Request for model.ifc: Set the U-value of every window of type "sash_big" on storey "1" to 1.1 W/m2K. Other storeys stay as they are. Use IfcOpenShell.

First a look at what the model holds.

```python
import ifcopenshell
import ifcopenshell.util.element

model = ifcopenshell.open("model.ifc")
print(model.schema)
storey = next(s for s in model.by_type("IfcBuildingStorey") if s.Name == "1")
windows = [e for e in ifcopenshell.util.element.get_decomposition(storey) if e.is_a("IfcWindow")]
seen = {}
for e in windows:
    element_type = ifcopenshell.util.element.get_type(e)
    key = (element_type.Name if element_type != e and element_type else None, ifcopenshell.util.element.get_pset(e, "Pset_WindowCommon", "ThermalTransmittance"))
    seen[key] = seen.get(key, 0) + 1
for (name, value), count in sorted(seen.items(), key=str):
    print(count, "x", name, "|", value)
```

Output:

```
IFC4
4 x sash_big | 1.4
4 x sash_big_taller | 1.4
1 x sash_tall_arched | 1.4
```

```python
import ifcopenshell
import ifcopenshell.api.pset
import ifcopenshell.util.element

model = ifcopenshell.open("model.ifc")

storey = next(s for s in model.by_type("IfcBuildingStorey") if s.Name == "1")
windows = [e for e in ifcopenshell.util.element.get_decomposition(storey) if e.is_a("IfcWindow")]

count = 0
for e in windows:
    element_type = ifcopenshell.util.element.get_type(e)
    if element_type in (None, e) or element_type.Name != "sash_big":
        continue
    # add_pset returns the element's existing set when there is one.
    pset = ifcopenshell.api.pset.add_pset(model, product=e, name="Pset_WindowCommon")
    ifcopenshell.api.pset.edit_pset(model, pset=pset, properties={"ThermalTransmittance": 1.1})
    count += 1

print(count, "windows updated")

model.write("model-out.ifc")
```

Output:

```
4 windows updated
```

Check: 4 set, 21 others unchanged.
